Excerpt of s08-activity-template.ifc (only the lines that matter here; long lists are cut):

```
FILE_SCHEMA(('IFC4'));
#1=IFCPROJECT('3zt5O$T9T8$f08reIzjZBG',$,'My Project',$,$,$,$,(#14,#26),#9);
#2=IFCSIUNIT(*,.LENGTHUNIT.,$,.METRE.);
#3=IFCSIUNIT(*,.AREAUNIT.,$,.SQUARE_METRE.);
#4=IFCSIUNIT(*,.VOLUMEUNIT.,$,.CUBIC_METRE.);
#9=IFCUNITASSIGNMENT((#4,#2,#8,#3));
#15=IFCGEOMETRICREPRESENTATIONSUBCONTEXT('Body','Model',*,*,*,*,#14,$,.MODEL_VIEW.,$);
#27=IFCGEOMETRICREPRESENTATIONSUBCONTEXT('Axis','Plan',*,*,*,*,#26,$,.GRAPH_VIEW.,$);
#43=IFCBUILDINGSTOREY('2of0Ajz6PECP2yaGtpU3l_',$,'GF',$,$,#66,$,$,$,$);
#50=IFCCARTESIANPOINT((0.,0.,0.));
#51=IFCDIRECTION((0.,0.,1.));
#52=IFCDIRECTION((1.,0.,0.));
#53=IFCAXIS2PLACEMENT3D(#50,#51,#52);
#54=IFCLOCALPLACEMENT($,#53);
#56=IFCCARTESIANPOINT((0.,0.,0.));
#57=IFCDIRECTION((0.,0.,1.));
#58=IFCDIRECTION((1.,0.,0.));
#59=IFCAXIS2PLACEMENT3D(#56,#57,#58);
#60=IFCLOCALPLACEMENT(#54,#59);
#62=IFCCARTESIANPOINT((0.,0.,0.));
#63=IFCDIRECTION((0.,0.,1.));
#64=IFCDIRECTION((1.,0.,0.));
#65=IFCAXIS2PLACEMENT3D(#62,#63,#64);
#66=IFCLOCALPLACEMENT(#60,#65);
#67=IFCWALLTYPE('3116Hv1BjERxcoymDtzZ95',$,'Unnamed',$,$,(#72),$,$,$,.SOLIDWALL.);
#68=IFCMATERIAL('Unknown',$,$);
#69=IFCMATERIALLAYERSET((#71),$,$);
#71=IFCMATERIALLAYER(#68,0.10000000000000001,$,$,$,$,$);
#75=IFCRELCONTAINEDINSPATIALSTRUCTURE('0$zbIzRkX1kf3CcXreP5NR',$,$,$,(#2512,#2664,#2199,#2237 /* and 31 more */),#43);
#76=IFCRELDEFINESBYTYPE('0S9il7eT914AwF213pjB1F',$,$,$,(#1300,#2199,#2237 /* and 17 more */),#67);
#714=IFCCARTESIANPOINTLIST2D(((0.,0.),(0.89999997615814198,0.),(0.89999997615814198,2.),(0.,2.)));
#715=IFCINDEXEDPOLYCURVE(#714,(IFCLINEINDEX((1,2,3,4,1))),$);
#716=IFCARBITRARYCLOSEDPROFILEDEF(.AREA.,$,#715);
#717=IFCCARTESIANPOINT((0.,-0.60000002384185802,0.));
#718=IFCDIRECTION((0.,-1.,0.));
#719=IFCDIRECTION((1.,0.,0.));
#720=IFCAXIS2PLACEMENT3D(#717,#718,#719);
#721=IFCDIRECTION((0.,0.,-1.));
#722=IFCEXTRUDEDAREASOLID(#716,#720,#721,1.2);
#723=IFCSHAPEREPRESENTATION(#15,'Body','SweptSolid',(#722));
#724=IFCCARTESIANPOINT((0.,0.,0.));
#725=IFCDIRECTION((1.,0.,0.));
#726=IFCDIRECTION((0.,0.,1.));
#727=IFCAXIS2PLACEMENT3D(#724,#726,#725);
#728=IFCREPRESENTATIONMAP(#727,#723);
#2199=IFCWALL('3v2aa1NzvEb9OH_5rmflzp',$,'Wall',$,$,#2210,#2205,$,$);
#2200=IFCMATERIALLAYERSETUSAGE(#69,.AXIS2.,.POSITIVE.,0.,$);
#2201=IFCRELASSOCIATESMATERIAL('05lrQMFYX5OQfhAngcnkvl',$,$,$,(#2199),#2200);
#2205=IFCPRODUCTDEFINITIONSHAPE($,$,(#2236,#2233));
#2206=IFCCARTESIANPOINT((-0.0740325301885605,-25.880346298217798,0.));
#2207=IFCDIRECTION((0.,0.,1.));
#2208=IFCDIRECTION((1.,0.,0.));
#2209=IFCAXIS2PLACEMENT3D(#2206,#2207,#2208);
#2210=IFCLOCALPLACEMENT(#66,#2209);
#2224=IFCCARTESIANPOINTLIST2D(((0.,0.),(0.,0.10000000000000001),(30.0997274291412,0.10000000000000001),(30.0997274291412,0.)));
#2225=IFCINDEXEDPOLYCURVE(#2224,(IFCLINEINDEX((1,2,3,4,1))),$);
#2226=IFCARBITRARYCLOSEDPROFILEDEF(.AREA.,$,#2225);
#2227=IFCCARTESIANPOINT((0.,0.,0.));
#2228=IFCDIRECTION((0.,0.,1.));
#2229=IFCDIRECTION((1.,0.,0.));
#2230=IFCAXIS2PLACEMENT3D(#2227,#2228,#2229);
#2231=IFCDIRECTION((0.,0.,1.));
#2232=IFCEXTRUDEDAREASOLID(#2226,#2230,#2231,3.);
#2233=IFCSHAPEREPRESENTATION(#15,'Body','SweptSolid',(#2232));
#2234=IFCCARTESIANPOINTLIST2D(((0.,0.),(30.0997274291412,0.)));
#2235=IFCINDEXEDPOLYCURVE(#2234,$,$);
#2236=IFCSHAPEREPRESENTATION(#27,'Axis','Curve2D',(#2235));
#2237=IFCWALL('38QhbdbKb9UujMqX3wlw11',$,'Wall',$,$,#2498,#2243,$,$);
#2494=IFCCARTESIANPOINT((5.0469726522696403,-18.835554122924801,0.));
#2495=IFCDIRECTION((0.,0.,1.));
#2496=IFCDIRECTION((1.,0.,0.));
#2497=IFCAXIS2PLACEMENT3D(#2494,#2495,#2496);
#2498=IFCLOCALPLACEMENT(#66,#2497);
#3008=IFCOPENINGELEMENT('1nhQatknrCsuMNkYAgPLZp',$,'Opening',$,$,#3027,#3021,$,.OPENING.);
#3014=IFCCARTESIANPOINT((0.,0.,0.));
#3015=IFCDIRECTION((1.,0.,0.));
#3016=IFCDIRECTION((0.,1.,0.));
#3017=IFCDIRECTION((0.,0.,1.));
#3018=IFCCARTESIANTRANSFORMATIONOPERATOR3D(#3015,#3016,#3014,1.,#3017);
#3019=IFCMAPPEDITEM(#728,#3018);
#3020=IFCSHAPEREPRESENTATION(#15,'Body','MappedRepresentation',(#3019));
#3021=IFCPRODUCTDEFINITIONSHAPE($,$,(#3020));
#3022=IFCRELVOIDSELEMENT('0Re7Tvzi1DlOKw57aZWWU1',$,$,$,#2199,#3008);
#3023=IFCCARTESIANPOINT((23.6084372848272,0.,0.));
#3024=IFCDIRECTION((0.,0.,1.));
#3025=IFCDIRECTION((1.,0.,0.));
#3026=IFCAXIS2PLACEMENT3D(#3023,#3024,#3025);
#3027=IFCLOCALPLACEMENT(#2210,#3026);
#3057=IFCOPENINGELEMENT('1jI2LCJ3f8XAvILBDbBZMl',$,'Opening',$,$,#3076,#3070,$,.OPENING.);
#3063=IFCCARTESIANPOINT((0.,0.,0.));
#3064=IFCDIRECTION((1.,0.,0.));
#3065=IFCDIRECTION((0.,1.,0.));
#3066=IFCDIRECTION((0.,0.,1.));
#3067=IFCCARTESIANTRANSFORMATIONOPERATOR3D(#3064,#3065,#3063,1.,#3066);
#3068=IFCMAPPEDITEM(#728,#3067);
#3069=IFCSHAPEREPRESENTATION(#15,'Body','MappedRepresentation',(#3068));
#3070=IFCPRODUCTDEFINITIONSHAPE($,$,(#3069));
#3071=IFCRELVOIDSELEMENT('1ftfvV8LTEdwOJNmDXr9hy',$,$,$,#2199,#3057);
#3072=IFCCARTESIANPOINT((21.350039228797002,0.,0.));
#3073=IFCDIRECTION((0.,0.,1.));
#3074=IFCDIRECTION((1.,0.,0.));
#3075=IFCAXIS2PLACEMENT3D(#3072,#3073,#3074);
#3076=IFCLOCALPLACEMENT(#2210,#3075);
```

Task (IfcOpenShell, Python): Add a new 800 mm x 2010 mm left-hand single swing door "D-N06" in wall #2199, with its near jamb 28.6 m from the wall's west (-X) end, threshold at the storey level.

```python
import numpy as np
import ifcopenshell
import ifcopenshell.api.feature
import ifcopenshell.api.geometry
import ifcopenshell.api.root
import ifcopenshell.api.spatial
import ifcopenshell.geom
import ifcopenshell.util.element
import ifcopenshell.util.placement
import ifcopenshell.util.representation
import ifcopenshell.util.shape
import ifcopenshell.util.unit

model = ifcopenshell.open("s08-activity-template.ifc")
unit_scale = ifcopenshell.util.unit.calculate_unit_scale(model)
settings = ifcopenshell.geom.settings()


def volume(element):
    """Net volume in cubic metres, openings subtracted."""
    shape = ifcopenshell.geom.create_shape(settings, element)
    return ifcopenshell.util.shape.get_volume(shape.geometry)


wall = model.by_id(2199)
storey = ifcopenshell.util.element.get_container(wall, ifc_class="IfcBuildingStorey")
context = ifcopenshell.util.representation.get_context(model, "Model", "Body", "MODEL_VIEW")
before = volume(wall)

width, height, from_end, sill = 0.8, 2.01, 28.6, 0.0  # metres

# The wall runs along its own X axis, and the end named is its -X end.
wall_shape = ifcopenshell.geom.create_shape(settings, wall)
x, y, z = ifcopenshell.util.shape.get_vertices(wall_shape.geometry).T
start = x.min() + from_end
face, thickness = float(y.min()), float(y.max() - y.min())
wall_matrix = ifcopenshell.util.placement.get_local_placement(wall.ObjectPlacement)
level = ifcopenshell.util.placement.get_local_placement(storey.ObjectPlacement)[2, 3]


def in_wall(x, y):
    """Placement at x, y metres in the wall's axes, at sill height."""
    matrix = wall_matrix.copy()
    matrix[:, 3] = wall_matrix @ np.array([x / unit_scale, y / unit_scale, 0.0, 1.0])
    matrix[2, 3] = level + sill / unit_scale
    return matrix


# Opening: a box that overshoots both wall faces by 50 mm.
opening = ifcopenshell.api.root.create_entity(model, ifc_class="IfcOpeningElement", predefined_type="OPENING")
box = ifcopenshell.api.geometry.add_wall_representation(
    model, context=context, length=width, height=height, thickness=thickness + 0.1
)
ifcopenshell.api.geometry.assign_representation(model, product=opening, representation=box)
ifcopenshell.api.geometry.edit_object_placement(model, product=opening, matrix=in_wall(start, face - 0.05), is_si=False)
ifcopenshell.api.feature.add_feature(model, feature=opening, element=wall)

door = ifcopenshell.api.root.create_entity(model, ifc_class="IfcDoor", name="D-N06", predefined_type="DOOR")
door.OverallWidth, door.OverallHeight = width / unit_scale, height / unit_scale
door.OperationType = "SINGLE_SWING_LEFT"
body = ifcopenshell.api.geometry.add_door_representation(
    model,
    context=context,
    overall_width=door.OverallWidth,
    overall_height=door.OverallHeight,
    operation_type="SINGLE_SWING_LEFT",
    lining_properties={"LiningDepth": thickness / unit_scale, "ThresholdDepth": thickness / unit_scale},
)
ifcopenshell.api.geometry.assign_representation(model, product=door, representation=body)
ifcopenshell.api.spatial.assign_container(model, products=[door], relating_structure=storey)
ifcopenshell.api.feature.add_filling(model, opening=opening, element=door)

# The lining spans the wall, so the door starts at the wall face.
ifcopenshell.api.geometry.edit_object_placement(model, product=door, matrix=in_wall(start, face), is_si=False)

after = volume(wall)

print(f"wall volume {before:.3f} -> {after:.3f} m3")

model.write("s08-activity-template_rev.ifc")
```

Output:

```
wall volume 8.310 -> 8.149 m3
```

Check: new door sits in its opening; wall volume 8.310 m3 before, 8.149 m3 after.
